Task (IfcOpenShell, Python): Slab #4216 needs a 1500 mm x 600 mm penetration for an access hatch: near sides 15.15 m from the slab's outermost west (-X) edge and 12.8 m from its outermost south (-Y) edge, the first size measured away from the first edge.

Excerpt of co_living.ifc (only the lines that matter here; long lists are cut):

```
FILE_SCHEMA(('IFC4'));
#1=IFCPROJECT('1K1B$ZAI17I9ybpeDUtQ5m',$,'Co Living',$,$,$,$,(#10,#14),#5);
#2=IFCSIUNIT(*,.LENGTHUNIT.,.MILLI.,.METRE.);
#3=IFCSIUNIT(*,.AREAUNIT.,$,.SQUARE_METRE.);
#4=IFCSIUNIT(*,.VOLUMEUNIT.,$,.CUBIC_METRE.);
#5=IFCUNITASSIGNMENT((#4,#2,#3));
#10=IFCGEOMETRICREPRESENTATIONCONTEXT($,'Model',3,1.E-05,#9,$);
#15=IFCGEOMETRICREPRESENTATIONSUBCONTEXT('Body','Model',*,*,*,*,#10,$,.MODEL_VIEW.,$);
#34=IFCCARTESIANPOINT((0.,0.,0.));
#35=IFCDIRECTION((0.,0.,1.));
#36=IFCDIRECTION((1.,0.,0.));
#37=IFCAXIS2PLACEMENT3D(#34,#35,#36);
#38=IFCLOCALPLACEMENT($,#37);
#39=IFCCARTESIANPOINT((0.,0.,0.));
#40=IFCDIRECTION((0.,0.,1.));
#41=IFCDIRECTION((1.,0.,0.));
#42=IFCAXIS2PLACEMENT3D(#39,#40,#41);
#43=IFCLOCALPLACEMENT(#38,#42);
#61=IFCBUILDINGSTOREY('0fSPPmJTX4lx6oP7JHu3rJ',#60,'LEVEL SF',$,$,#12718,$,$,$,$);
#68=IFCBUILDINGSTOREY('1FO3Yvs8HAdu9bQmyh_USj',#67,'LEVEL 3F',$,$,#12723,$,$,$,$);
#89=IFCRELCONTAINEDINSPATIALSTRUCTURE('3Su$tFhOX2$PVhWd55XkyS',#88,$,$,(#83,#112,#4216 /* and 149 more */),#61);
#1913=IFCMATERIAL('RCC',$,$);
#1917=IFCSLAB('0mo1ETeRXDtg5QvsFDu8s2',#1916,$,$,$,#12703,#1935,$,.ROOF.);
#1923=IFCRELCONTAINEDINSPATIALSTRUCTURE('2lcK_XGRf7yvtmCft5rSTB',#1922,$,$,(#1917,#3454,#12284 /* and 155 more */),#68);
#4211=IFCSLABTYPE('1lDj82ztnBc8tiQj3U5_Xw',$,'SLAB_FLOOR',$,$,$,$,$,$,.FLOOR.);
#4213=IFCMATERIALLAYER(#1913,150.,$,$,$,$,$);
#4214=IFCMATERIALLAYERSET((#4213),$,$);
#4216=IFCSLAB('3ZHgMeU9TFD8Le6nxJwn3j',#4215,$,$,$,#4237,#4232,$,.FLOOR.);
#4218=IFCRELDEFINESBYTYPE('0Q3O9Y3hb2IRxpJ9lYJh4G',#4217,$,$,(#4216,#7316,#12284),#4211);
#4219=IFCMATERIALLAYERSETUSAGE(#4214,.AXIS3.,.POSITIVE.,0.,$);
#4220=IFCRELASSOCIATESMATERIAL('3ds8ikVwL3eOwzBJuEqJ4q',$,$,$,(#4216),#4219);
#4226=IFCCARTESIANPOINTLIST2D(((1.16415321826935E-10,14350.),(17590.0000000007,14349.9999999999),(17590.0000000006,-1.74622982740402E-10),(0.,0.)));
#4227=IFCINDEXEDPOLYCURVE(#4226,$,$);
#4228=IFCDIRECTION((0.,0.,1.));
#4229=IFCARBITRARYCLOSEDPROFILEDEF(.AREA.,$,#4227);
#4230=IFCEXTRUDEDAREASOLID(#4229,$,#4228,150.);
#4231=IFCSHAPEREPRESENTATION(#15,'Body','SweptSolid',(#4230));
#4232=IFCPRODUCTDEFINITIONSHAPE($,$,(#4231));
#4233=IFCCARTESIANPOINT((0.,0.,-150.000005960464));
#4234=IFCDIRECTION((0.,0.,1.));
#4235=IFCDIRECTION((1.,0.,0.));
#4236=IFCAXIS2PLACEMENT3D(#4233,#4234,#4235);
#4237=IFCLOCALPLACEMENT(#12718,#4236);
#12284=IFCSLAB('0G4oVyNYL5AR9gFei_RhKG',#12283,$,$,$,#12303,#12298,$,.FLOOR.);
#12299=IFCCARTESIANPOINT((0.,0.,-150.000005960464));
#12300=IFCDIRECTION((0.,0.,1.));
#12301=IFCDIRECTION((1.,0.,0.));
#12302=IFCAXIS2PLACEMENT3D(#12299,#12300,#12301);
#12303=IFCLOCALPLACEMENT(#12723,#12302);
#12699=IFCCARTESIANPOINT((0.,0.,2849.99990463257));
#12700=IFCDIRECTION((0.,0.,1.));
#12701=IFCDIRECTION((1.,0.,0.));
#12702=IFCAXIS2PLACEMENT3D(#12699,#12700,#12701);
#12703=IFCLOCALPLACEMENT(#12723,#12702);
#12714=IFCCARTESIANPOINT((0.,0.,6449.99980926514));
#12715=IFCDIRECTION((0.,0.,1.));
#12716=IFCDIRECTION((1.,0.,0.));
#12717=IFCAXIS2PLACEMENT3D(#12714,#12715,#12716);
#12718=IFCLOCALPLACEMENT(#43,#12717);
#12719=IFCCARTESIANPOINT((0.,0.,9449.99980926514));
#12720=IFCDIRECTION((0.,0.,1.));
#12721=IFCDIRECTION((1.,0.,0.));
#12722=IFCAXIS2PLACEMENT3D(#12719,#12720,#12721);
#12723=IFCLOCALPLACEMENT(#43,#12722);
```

```python
import numpy as np
import ifcopenshell
import ifcopenshell.api.feature
import ifcopenshell.api.geometry
import ifcopenshell.api.root
import ifcopenshell.geom
import ifcopenshell.util.placement
import ifcopenshell.util.representation
import ifcopenshell.util.shape
import ifcopenshell.util.unit

model = ifcopenshell.open("co_living.ifc")
unit_scale = ifcopenshell.util.unit.calculate_unit_scale(model)
settings = ifcopenshell.geom.settings()


def volume(element):
    """Net volume in cubic metres, openings subtracted."""
    shape = ifcopenshell.geom.create_shape(settings, element)
    return ifcopenshell.util.shape.get_volume(shape.geometry)


slab = model.by_guid("3ZHgMeU9TFD8Le6nxJwn3j")
before = volume(slab)

# Extent in the slab's own axes, in metres. The edges named are its -X and -Y sides.
slab_shape = ifcopenshell.geom.create_shape(settings, slab)
vertices = ifcopenshell.util.shape.get_vertices(slab_shape.geometry)
x_min, y_min, bottom = vertices.min(axis=0)
top = vertices[:, 2].max()

opening = ifcopenshell.api.root.create_entity(model, ifc_class="IfcOpeningElement", name="Access hatch opening", predefined_type="OPENING")
context = ifcopenshell.util.representation.get_context(model, "Model", "Body", "MODEL_VIEW")
width, depth = 1.5, 0.6
outline = [(0.0, 0.0), (width, 0.0), (width, depth), (0.0, depth), (0.0, 0.0)]
# Overshoot both faces by 50 mm so the cut is clean.
shape = ifcopenshell.api.geometry.add_slab_representation(
    model, context=context, depth=top - bottom + 0.1, polyline=outline
)
ifcopenshell.api.geometry.assign_representation(model, product=opening, representation=shape)

matrix = ifcopenshell.util.placement.get_local_placement(slab.ObjectPlacement)
matrix[:, 3] = matrix @ np.append(np.array([x_min + 15.15, y_min + 12.8, bottom - 0.05]) / unit_scale, 1.0)
ifcopenshell.api.geometry.edit_object_placement(model, product=opening, matrix=matrix, is_si=False)
ifcopenshell.api.feature.add_feature(model, feature=opening, element=slab)

after = volume(slab)

print(f"slab volume {before:.3f} -> {after:.3f} m3")

model.write("co_living_updated.ifc")
```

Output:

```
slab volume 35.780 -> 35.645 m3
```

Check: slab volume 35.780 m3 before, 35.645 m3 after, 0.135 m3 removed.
